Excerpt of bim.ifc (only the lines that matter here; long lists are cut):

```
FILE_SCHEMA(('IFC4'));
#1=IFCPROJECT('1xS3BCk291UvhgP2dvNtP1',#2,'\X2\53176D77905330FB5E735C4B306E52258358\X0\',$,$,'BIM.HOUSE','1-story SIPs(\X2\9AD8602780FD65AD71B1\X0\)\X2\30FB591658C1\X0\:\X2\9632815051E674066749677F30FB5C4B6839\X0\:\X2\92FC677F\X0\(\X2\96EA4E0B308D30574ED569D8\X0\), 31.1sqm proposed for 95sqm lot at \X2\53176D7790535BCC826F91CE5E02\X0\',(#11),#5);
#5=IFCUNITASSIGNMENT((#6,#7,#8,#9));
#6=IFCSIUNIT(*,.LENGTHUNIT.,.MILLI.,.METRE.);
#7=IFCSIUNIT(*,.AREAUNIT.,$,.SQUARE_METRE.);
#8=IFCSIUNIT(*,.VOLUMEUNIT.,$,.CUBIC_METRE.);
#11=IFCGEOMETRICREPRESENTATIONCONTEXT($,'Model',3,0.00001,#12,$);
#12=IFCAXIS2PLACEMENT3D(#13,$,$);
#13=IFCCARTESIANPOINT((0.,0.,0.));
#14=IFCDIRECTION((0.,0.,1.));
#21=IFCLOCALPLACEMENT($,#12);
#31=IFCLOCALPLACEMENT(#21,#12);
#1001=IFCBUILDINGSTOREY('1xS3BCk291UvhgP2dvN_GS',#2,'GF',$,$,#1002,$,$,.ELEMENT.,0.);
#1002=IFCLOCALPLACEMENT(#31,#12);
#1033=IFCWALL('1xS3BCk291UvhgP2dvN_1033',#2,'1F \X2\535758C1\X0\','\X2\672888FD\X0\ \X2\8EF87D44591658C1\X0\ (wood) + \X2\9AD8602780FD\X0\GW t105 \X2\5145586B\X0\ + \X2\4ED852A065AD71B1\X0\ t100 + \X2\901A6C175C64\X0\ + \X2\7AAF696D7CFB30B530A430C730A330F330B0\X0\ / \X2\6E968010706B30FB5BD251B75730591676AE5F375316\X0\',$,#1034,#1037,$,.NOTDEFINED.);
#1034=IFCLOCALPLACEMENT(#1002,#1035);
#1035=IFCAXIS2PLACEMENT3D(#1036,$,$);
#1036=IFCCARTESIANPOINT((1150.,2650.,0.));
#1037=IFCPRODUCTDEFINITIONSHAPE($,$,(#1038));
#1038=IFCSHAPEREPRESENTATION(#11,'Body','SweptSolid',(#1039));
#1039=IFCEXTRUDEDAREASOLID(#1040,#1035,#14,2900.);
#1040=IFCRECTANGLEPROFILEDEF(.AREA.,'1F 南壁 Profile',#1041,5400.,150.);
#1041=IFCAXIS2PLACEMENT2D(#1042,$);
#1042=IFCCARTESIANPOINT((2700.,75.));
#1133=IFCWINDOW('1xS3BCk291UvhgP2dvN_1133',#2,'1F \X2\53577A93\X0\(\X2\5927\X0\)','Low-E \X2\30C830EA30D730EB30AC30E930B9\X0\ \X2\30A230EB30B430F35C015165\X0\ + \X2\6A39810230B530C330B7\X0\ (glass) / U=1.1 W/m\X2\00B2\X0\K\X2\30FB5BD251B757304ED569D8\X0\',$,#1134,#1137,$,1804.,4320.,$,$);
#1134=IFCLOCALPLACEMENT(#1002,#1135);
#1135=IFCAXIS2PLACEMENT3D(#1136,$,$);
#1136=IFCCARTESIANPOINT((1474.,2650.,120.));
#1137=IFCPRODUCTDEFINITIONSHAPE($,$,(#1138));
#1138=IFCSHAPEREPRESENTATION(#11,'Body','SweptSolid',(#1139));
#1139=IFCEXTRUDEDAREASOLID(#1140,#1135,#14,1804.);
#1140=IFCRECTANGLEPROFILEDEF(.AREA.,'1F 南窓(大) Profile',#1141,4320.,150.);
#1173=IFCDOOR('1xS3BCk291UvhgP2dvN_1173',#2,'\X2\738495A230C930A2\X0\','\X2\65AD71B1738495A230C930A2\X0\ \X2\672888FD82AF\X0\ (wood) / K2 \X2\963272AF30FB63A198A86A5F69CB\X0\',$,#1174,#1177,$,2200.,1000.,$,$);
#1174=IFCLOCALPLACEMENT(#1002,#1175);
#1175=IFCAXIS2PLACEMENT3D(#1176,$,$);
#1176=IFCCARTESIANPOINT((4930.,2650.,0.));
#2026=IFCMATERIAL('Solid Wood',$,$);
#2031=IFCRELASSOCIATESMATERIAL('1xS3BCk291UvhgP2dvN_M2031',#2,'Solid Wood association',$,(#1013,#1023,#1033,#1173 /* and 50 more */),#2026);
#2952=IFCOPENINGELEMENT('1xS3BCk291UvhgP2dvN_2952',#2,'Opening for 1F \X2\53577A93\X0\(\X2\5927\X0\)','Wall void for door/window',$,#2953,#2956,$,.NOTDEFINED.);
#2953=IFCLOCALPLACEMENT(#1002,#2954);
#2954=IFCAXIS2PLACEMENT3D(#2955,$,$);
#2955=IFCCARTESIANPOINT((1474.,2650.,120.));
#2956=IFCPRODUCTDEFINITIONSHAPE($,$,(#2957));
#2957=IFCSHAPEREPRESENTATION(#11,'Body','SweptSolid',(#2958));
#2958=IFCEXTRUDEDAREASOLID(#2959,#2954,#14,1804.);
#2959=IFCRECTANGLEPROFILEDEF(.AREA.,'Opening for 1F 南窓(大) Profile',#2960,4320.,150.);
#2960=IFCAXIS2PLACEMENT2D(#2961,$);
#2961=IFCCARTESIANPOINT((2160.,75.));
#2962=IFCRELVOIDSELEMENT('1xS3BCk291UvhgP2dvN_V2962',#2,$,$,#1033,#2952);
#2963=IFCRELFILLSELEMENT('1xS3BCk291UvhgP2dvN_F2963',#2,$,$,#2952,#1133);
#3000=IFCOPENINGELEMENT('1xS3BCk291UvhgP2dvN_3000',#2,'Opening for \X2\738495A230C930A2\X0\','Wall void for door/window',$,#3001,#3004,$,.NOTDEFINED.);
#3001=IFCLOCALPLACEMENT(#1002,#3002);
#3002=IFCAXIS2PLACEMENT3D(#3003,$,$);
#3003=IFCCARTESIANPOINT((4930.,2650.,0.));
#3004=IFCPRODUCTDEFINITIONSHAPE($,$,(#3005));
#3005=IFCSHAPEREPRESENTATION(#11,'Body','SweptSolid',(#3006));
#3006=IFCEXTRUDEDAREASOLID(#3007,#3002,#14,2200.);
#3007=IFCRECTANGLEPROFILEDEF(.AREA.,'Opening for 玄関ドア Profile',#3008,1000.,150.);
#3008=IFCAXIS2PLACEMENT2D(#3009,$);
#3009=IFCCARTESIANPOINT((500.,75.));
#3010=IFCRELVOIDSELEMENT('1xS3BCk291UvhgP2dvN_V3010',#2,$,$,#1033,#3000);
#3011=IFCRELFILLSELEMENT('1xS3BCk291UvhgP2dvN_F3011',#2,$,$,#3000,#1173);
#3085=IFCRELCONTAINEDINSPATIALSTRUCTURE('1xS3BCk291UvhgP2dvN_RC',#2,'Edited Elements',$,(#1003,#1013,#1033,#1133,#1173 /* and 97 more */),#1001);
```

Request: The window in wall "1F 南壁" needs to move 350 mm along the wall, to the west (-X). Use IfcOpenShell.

```python
import ifcopenshell
import ifcopenshell.api.geometry
import ifcopenshell.util.placement

model = ifcopenshell.open("bim.ifc")

window = model.by_guid("1xS3BCk291UvhgP2dvN_1133")
opening = window.FillsVoids[0].RelatingOpeningElement
wall = opening.VoidsElements[0].RelatingBuildingElement

wall_matrix = ifcopenshell.util.placement.get_local_placement(wall.ObjectPlacement)
shift = wall_matrix[:3, 0] * -350.0
before = ifcopenshell.util.placement.get_local_placement(window.ObjectPlacement)[:3, 3].copy()

# The window is not placed relative to its opening, so move both.
for product in (opening, window):
    matrix = ifcopenshell.util.placement.get_local_placement(product.ObjectPlacement)
    matrix[:3, 3] += shift
    ifcopenshell.api.geometry.edit_object_placement(model, product=product, matrix=matrix, is_si=False)

after = ifcopenshell.util.placement.get_local_placement(window.ObjectPlacement)[:3, 3]
print("window moved by", (after - before).round(3) + 0.0)

model.write("bim_edited.ifc")
```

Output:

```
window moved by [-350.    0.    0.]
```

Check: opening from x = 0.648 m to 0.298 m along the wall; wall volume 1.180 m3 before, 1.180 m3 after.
